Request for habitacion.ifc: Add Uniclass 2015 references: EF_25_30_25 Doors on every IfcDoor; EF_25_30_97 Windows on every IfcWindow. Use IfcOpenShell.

First a look at what the model holds.

```python
import ifcopenshell

model = ifcopenshell.open("habitacion.ifc")
print(model.schema)
print("classifications:", [c.Name for c in model.by_type("IfcClassification")])
for ifc_class in ("IfcDoor", "IfcRoof", "IfcStair", "IfcWall", "IfcWindow"):
    print(ifc_class, len(model.by_type(ifc_class)))
```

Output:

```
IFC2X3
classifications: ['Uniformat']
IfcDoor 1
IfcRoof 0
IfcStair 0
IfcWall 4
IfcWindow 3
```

```python
import ifcopenshell
import ifcopenshell.api.classification

model = ifcopenshell.open("habitacion.ifc")

# IFC2X3 requires Source and Edition and has no link from the project to the system.
system = model.create_entity("IfcClassification", Source="NBS", Edition="2015", Name="Uniclass 2015")

codes = {
    "IfcDoor": ("EF_25_30_25", "Doors"),
    "IfcWindow": ("EF_25_30_97", "Windows"),
}
for ifc_class, (code, name) in codes.items():
    products = model.by_type(ifc_class)
    ifcopenshell.api.classification.add_reference(
        model, products=products, classification=system, identification=code, name=name
    )
    print(code, len(products))

model.write("habitacion_v2.ifc")
```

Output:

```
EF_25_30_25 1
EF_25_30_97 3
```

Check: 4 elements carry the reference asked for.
